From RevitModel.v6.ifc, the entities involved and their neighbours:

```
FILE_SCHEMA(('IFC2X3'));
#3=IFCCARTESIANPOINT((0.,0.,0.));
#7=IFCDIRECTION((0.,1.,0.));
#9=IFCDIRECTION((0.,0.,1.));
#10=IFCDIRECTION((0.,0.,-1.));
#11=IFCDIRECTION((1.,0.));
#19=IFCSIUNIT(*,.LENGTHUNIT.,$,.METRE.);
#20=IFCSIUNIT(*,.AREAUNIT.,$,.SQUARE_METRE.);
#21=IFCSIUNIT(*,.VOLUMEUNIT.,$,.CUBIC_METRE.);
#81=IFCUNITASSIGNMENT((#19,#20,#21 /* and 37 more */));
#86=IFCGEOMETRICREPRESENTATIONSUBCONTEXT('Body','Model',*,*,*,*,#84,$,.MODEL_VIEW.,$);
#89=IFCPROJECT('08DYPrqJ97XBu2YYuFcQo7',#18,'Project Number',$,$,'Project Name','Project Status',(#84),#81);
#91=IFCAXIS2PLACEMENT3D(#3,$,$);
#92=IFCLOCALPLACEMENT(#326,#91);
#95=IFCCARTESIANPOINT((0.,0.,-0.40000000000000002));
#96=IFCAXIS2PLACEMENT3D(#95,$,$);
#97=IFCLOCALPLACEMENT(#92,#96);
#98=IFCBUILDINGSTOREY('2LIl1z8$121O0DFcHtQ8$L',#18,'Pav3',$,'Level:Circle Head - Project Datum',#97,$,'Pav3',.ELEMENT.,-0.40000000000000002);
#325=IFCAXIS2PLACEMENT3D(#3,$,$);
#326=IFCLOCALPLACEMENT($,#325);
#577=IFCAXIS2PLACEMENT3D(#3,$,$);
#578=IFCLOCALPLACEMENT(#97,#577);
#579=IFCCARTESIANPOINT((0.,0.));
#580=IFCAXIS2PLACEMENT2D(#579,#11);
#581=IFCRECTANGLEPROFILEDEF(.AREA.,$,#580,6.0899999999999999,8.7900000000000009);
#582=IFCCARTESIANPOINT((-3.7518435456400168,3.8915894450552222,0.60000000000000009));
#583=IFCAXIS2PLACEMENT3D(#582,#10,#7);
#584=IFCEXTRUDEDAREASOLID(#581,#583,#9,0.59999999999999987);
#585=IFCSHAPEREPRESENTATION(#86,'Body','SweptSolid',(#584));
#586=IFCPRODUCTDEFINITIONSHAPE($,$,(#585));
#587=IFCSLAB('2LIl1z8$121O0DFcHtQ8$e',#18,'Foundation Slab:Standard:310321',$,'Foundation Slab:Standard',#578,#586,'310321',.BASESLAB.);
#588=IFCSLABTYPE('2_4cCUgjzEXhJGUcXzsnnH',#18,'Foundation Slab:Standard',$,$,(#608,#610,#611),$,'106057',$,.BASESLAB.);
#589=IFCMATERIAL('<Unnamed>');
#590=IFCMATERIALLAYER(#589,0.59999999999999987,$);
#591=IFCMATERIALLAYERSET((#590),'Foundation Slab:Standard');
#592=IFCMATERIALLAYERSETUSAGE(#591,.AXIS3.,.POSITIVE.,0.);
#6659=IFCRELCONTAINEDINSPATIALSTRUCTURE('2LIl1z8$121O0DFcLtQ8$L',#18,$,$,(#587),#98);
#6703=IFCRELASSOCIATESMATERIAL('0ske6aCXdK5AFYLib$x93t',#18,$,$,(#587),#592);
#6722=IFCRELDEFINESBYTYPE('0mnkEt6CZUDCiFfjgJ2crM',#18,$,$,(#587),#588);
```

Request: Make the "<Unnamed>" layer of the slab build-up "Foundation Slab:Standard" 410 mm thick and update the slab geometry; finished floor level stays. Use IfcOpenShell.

```python
import ifcopenshell
import ifcopenshell.util.element
import ifcopenshell.util.representation
import ifcopenshell.util.unit

model = ifcopenshell.open("RevitModel.v6.ifc")
unit_scale = ifcopenshell.util.unit.calculate_unit_scale(model)

layer_set = model.by_id(591)
layer = next(l for l in layer_set.MaterialLayers if l.Material and l.Material.Name == "<Unnamed>")
change = 0.41 / unit_scale - layer.LayerThickness
layer.LayerThickness += change

# Geometry does not follow the layer set by itself.
slabs = [e for e in ifcopenshell.util.element.get_elements_by_material(model, layer_set) if e.is_a("IfcSlab")]
for slab in sorted(slabs, key=lambda e: e.id()):
    body = ifcopenshell.util.representation.get_representation(slab, "Model", "Body")
    solid = body.Items[0]
    old_depth = solid.Depth
    solid.Depth += change
    print(slab.id(), f"{old_depth:g} -> {solid.Depth:g}")

# The layers are counted up from the underside, which has moved.
for usage in {ifcopenshell.util.element.get_material(slab) for slab in slabs}:
    usage.OffsetFromReferenceLine -= change

model.write("RevitModel.v6_v2.ifc")
```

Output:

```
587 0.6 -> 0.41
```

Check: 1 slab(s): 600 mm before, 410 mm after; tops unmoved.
